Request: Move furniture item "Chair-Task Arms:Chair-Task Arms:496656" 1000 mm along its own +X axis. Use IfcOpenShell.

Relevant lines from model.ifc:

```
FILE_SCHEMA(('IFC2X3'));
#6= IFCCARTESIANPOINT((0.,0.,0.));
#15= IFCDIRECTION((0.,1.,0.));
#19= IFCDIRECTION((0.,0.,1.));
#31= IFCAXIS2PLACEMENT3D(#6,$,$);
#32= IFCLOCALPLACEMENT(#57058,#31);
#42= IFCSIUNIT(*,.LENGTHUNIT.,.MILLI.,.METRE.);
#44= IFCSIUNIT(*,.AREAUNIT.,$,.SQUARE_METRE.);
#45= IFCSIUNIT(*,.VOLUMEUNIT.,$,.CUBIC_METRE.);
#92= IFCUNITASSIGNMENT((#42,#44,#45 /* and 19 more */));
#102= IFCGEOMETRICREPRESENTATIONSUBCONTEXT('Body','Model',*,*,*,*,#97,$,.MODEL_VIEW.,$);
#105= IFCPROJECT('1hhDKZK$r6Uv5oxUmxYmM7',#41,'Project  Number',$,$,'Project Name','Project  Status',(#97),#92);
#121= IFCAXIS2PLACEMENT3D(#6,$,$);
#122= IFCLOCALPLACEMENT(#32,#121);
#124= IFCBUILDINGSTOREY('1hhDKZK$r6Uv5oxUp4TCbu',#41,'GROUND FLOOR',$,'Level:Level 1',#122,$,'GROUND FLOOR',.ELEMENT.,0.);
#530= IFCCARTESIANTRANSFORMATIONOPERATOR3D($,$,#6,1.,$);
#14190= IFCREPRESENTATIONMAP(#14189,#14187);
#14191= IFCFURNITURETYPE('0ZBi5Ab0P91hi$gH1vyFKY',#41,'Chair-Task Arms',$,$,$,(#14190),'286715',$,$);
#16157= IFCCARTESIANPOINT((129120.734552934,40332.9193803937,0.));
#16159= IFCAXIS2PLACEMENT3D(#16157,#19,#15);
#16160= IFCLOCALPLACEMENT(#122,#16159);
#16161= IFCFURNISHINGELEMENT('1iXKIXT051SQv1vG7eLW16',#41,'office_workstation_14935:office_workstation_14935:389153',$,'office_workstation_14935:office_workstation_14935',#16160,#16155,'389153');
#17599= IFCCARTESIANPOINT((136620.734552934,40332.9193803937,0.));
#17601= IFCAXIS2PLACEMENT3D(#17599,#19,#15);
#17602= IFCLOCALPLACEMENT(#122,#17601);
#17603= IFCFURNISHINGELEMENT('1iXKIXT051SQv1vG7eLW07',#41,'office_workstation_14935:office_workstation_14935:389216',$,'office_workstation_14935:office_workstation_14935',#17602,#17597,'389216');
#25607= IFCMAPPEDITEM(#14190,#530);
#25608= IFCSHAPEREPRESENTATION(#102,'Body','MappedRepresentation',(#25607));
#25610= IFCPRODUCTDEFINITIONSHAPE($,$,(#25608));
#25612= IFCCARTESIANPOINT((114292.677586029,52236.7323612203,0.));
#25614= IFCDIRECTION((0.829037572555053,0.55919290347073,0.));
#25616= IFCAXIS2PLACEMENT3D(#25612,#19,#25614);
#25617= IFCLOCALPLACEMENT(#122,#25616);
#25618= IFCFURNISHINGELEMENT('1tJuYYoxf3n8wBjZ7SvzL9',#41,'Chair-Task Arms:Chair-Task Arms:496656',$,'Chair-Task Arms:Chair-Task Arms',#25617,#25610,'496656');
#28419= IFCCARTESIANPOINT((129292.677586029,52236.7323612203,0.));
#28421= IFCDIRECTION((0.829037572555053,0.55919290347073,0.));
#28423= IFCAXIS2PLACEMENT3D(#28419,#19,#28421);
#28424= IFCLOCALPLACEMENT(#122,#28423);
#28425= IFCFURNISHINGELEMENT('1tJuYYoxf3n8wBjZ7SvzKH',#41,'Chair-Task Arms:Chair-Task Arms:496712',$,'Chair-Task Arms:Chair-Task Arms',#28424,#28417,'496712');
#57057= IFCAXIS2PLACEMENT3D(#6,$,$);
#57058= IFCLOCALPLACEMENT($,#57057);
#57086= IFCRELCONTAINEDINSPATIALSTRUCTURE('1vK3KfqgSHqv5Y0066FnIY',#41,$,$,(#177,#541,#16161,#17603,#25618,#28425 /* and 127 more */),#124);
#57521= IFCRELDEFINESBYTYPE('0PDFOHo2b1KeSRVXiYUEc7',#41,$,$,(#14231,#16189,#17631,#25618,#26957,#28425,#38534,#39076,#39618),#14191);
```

```python
import ifcopenshell
import ifcopenshell.api.geometry
import ifcopenshell.util.placement
import ifcopenshell.util.unit

model = ifcopenshell.open("model.ifc")
unit_scale = ifcopenshell.util.unit.calculate_unit_scale(model)

item = model.by_guid("1tJuYYoxf3n8wBjZ7SvzL9")
matrix = ifcopenshell.util.placement.get_local_placement(item.ObjectPlacement)
matrix[:3, 3] += matrix[:3, 0] * 1 / unit_scale
ifcopenshell.api.geometry.edit_object_placement(model, product=item, matrix=matrix, is_si=False)

print(ifcopenshell.util.placement.get_local_placement(item.ObjectPlacement).round(3) + 0.0)

model.write("model-out.ifc")
```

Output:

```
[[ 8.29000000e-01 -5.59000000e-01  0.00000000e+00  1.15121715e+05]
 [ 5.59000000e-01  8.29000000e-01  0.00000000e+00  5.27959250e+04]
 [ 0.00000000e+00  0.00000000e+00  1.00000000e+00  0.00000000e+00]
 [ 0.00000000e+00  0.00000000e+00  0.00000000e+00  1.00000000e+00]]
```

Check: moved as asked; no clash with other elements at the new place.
